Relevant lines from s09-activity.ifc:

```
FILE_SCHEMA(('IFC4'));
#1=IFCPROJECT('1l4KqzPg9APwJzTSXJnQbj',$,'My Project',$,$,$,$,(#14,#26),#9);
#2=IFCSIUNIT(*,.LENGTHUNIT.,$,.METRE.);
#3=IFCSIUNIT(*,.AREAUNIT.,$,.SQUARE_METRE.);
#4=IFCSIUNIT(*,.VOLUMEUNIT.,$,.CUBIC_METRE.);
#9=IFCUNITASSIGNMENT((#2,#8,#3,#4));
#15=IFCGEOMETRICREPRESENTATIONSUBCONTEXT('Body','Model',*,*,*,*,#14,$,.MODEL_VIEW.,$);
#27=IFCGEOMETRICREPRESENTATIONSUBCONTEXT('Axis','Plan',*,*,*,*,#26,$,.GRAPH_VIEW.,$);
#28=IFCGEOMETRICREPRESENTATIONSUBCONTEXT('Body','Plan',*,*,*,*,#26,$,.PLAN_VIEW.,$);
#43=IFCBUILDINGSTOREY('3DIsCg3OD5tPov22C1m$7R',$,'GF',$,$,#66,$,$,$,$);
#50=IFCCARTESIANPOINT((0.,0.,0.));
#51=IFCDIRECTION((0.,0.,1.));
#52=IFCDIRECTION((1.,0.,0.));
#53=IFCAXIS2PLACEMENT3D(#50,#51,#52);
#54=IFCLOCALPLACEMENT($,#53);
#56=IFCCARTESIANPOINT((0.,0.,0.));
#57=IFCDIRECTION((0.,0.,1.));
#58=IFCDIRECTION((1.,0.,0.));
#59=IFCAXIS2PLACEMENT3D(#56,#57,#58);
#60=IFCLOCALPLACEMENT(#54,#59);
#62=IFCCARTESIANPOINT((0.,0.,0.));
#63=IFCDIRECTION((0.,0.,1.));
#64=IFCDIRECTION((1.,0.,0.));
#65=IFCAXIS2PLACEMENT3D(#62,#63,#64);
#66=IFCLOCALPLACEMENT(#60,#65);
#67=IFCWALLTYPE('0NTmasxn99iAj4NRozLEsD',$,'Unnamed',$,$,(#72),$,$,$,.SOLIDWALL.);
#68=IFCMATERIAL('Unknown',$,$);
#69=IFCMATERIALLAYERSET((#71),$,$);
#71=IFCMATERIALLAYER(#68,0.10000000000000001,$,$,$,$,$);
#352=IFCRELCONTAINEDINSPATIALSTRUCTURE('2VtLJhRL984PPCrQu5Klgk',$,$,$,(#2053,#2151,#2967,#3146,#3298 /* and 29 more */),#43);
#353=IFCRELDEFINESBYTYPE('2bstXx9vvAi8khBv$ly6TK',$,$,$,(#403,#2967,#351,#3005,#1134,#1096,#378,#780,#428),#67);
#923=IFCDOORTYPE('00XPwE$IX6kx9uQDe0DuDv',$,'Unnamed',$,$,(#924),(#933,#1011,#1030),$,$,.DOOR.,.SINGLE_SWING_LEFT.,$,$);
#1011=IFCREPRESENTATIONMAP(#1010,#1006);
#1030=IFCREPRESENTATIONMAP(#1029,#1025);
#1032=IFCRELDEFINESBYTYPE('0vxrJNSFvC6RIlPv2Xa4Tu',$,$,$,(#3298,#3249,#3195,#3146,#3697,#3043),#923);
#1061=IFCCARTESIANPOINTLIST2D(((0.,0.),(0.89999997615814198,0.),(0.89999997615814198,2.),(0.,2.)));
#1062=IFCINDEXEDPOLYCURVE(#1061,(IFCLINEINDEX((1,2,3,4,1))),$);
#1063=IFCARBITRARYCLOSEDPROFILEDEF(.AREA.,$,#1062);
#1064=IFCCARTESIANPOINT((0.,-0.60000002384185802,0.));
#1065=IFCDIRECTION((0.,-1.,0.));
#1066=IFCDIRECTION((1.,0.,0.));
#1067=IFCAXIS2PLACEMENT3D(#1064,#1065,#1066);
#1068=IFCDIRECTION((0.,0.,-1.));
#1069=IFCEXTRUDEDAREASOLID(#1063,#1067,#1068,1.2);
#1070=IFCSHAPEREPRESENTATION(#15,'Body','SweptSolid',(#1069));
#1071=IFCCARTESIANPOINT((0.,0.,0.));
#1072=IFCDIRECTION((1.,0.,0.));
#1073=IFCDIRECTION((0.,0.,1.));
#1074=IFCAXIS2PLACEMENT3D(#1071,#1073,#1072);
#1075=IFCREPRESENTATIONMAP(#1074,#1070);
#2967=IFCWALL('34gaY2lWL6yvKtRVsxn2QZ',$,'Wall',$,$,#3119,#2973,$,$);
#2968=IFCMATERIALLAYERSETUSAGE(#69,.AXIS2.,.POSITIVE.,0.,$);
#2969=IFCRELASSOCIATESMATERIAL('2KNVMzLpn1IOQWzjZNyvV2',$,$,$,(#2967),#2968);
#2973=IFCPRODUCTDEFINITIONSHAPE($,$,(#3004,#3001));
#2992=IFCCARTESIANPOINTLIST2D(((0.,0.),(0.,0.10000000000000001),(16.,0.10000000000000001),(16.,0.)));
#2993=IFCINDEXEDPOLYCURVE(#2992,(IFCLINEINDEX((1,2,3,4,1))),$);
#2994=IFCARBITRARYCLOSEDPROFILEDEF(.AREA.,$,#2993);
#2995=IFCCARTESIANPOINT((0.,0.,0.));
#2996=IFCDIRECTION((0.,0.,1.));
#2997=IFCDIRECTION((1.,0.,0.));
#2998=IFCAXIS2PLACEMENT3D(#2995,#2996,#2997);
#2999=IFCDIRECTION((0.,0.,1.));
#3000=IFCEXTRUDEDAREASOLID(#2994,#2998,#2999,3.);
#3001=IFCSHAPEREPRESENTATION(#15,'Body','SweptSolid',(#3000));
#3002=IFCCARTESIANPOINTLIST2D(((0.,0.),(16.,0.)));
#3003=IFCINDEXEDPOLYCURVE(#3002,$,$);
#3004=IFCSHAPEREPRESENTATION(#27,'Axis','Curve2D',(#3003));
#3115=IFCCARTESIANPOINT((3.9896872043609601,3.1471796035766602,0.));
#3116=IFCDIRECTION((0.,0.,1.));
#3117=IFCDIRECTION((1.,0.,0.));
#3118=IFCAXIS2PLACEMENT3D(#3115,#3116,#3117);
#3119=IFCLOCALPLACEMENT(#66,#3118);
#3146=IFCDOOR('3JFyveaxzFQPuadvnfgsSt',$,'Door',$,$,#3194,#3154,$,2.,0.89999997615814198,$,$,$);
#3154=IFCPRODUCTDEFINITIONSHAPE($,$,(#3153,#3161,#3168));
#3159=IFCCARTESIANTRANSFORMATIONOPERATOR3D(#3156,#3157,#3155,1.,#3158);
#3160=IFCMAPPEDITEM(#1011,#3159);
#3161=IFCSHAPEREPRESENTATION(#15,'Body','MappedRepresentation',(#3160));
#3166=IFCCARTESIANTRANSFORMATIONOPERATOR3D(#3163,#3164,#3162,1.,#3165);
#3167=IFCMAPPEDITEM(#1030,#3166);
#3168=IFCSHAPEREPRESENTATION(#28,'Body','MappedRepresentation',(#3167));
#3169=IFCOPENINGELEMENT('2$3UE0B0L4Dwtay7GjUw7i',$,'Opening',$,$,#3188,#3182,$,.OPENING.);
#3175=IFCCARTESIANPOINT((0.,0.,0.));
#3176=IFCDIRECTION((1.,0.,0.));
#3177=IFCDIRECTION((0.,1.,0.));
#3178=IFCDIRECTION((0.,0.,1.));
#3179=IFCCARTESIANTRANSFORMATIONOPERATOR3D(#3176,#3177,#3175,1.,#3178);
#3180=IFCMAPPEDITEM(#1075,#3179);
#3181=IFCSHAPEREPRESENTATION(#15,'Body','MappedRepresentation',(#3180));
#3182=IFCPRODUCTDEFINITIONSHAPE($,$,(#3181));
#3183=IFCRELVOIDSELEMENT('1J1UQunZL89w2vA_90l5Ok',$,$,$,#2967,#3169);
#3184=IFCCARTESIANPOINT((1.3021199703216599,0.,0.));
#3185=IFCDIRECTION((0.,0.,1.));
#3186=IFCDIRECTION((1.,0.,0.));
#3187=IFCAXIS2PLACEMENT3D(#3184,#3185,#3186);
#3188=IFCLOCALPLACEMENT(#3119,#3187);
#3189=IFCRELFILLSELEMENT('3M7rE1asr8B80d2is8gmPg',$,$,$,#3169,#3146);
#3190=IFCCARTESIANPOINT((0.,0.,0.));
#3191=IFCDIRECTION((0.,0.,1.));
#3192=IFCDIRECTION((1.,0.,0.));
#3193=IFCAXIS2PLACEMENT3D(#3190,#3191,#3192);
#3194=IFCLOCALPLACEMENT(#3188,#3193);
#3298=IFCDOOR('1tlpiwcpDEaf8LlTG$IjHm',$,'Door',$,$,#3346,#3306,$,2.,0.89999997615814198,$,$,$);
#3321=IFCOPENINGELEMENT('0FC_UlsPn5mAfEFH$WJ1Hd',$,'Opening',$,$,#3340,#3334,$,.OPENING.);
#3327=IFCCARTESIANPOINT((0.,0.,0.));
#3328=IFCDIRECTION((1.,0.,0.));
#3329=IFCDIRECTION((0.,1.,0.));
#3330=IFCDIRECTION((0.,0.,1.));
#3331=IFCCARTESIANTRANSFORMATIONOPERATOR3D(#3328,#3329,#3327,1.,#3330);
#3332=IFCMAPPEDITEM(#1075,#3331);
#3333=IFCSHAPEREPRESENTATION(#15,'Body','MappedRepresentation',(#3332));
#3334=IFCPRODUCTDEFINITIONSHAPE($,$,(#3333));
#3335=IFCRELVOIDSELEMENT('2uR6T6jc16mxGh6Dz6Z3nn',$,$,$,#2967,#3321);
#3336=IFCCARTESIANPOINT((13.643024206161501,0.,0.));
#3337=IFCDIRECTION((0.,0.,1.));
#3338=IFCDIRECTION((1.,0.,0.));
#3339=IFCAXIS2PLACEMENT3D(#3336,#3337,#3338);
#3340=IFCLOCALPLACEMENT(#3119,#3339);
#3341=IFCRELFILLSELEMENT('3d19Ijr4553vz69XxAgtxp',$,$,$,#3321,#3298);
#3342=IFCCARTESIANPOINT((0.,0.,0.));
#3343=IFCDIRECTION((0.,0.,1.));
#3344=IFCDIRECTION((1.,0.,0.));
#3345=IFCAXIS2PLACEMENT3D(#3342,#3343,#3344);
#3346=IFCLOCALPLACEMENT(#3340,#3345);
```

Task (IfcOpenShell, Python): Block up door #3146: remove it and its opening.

```python
import ifcopenshell
import ifcopenshell.api.feature
import ifcopenshell.api.root
import ifcopenshell.geom
import ifcopenshell.util.shape

model = ifcopenshell.open("s09-activity.ifc")
settings = ifcopenshell.geom.settings()


def volume(element):
    """Net volume in cubic metres, openings subtracted."""
    shape = ifcopenshell.geom.create_shape(settings, element)
    return ifcopenshell.util.shape.get_volume(shape.geometry)


door = model.by_id(3146)
opening = door.FillsVoids[0].RelatingOpeningElement
wall = opening.VoidsElements[0].RelatingBuildingElement
before = volume(wall)

ifcopenshell.api.root.remove_product(model, product=door)
ifcopenshell.api.feature.remove_feature(model, feature=opening)

after = volume(wall)

print(f"wall volume {before:.3f} -> {after:.3f} m3")

model.write("s09-activity-out.ifc")
```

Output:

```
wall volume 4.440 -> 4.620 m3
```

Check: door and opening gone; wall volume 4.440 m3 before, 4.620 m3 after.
